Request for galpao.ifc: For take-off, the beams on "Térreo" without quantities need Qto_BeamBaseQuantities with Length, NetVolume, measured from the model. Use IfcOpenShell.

First a look at what the model holds.

```python
import ifcopenshell
import ifcopenshell.util.element
import ifcopenshell.util.unit

model = ifcopenshell.open("galpao.ifc")
print(model.schema)
for unit_type in ("LENGTHUNIT", "AREAUNIT", "VOLUMEUNIT"):
    print(unit_type, ifcopenshell.util.unit.calculate_unit_scale(model, unit_type))
storey = next(s for s in model.by_type("IfcBuildingStorey") if s.Name == "Térreo")
beams = [e for e in ifcopenshell.util.element.get_decomposition(storey) if e.is_a("IfcBeam")]
for e in sorted(beams, key=lambda e: e.id()):
    print(e.id(), e.is_a(), e.Name, list(ifcopenshell.util.element.get_psets(e, qtos_only=True)), sep=" | ")
```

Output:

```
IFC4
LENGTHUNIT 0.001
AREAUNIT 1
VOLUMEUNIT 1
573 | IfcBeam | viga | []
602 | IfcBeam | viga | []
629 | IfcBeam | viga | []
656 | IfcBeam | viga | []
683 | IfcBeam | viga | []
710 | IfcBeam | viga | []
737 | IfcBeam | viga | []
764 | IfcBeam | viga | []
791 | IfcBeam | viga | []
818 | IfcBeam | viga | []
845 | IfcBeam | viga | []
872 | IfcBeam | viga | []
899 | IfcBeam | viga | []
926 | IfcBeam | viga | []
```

```python
import ifcopenshell
import ifcopenshell.api.pset
import ifcopenshell.geom
import ifcopenshell.util.element
import ifcopenshell.util.shape
import ifcopenshell.util.unit

model = ifcopenshell.open("galpao.ifc")
unit_scale = ifcopenshell.util.unit.calculate_unit_scale(model)
volume_scale = ifcopenshell.util.unit.calculate_unit_scale(model, "VOLUMEUNIT")
settings = ifcopenshell.geom.settings()

storey = next(s for s in model.by_type("IfcBuildingStorey") if s.Name == "Térreo")
beams = [e for e in ifcopenshell.util.element.get_decomposition(storey) if e.is_a("IfcBeam")]

for e in sorted(beams, key=lambda e: e.id()):
    if ifcopenshell.util.element.get_psets(e, qtos_only=True, should_inherit=False):
        continue
    # Geometry comes back in metres, in the element's own axes.
    shape = ifcopenshell.geom.create_shape(settings, e)
    values = {
        "Length": ifcopenshell.util.shape.get_max_xyz(shape.geometry) / unit_scale,
        "NetVolume": ifcopenshell.util.shape.get_volume(shape.geometry) / volume_scale,
    }
    qto = ifcopenshell.api.pset.add_qto(model, product=e, name="Qto_BeamBaseQuantities")
    ifcopenshell.api.pset.edit_qto(model, qto=qto, properties=values)
    print(e.id(), {k: round(v, 3) for k, v in values.items()})

model.write("galpao_v2.ifc")
```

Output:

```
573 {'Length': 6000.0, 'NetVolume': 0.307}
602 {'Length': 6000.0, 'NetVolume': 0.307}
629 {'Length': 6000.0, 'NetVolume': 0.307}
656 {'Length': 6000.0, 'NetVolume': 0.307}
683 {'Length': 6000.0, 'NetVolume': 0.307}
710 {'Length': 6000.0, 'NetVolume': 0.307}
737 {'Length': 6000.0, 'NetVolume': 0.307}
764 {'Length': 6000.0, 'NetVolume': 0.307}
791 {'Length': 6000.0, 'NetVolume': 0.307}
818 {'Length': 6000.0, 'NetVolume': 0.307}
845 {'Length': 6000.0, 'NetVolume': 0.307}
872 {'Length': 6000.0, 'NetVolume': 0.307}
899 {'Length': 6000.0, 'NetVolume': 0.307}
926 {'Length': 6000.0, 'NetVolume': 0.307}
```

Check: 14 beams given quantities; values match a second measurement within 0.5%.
